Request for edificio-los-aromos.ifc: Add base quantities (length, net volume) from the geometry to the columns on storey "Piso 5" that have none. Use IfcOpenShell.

First a look at what the model holds.

```python
import ifcopenshell
import ifcopenshell.util.element
import ifcopenshell.util.unit

model = ifcopenshell.open("edificio-los-aromos.ifc")
print(model.schema)
for unit_type in ("LENGTHUNIT", "AREAUNIT", "VOLUMEUNIT"):
    print(unit_type, ifcopenshell.util.unit.calculate_unit_scale(model, unit_type))
storey = next(s for s in model.by_type("IfcBuildingStorey") if s.Name == "Piso 5")
columns = [e for e in ifcopenshell.util.element.get_decomposition(storey) if e.is_a("IfcColumn")]
for e in sorted(columns, key=lambda e: e.id()):
    print(e.id(), e.is_a(), e.Name, list(ifcopenshell.util.element.get_psets(e, qtos_only=True)), sep=" | ")
```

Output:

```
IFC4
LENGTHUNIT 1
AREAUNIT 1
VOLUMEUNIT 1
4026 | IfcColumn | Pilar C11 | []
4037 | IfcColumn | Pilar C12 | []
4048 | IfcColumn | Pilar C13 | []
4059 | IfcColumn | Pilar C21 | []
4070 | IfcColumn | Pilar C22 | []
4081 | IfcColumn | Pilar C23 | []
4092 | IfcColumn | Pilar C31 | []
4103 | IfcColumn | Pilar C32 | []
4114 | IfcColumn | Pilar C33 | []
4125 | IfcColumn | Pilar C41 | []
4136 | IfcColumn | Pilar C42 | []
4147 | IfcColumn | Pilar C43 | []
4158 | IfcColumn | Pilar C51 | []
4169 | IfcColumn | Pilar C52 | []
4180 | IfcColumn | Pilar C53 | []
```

```python
import ifcopenshell
import ifcopenshell.api.pset
import ifcopenshell.geom
import ifcopenshell.util.element
import ifcopenshell.util.shape
import ifcopenshell.util.unit

model = ifcopenshell.open("edificio-los-aromos.ifc")
unit_scale = ifcopenshell.util.unit.calculate_unit_scale(model)
volume_scale = ifcopenshell.util.unit.calculate_unit_scale(model, "VOLUMEUNIT")
settings = ifcopenshell.geom.settings()

storey = next(s for s in model.by_type("IfcBuildingStorey") if s.Name == "Piso 5")
columns = [e for e in ifcopenshell.util.element.get_decomposition(storey) if e.is_a("IfcColumn")]

for e in sorted(columns, key=lambda e: e.id()):
    if ifcopenshell.util.element.get_psets(e, qtos_only=True, should_inherit=False):
        continue
    # Geometry comes back in metres, in the element's own axes.
    shape = ifcopenshell.geom.create_shape(settings, e)
    values = {
        "Length": ifcopenshell.util.shape.get_z(shape.geometry) / unit_scale,
        "NetVolume": ifcopenshell.util.shape.get_volume(shape.geometry) / volume_scale,
    }
    qto = ifcopenshell.api.pset.add_qto(model, product=e, name="Qto_ColumnBaseQuantities")
    ifcopenshell.api.pset.edit_qto(model, qto=qto, properties=values)
    print(e.id(), {k: round(v, 3) for k, v in values.items()})

model.write("edificio-los-aromos-out.ifc")
```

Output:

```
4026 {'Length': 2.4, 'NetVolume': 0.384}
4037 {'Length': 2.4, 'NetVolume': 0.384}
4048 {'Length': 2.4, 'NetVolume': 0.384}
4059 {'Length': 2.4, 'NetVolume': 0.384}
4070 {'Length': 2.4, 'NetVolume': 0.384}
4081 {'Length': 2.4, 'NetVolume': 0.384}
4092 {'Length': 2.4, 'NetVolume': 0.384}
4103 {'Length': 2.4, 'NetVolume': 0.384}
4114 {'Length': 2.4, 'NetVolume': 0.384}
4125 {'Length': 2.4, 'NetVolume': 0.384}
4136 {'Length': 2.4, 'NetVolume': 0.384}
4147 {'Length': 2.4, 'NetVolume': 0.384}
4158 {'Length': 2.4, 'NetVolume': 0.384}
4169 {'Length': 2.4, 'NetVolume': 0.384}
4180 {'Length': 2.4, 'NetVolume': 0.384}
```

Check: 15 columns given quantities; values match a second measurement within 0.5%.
